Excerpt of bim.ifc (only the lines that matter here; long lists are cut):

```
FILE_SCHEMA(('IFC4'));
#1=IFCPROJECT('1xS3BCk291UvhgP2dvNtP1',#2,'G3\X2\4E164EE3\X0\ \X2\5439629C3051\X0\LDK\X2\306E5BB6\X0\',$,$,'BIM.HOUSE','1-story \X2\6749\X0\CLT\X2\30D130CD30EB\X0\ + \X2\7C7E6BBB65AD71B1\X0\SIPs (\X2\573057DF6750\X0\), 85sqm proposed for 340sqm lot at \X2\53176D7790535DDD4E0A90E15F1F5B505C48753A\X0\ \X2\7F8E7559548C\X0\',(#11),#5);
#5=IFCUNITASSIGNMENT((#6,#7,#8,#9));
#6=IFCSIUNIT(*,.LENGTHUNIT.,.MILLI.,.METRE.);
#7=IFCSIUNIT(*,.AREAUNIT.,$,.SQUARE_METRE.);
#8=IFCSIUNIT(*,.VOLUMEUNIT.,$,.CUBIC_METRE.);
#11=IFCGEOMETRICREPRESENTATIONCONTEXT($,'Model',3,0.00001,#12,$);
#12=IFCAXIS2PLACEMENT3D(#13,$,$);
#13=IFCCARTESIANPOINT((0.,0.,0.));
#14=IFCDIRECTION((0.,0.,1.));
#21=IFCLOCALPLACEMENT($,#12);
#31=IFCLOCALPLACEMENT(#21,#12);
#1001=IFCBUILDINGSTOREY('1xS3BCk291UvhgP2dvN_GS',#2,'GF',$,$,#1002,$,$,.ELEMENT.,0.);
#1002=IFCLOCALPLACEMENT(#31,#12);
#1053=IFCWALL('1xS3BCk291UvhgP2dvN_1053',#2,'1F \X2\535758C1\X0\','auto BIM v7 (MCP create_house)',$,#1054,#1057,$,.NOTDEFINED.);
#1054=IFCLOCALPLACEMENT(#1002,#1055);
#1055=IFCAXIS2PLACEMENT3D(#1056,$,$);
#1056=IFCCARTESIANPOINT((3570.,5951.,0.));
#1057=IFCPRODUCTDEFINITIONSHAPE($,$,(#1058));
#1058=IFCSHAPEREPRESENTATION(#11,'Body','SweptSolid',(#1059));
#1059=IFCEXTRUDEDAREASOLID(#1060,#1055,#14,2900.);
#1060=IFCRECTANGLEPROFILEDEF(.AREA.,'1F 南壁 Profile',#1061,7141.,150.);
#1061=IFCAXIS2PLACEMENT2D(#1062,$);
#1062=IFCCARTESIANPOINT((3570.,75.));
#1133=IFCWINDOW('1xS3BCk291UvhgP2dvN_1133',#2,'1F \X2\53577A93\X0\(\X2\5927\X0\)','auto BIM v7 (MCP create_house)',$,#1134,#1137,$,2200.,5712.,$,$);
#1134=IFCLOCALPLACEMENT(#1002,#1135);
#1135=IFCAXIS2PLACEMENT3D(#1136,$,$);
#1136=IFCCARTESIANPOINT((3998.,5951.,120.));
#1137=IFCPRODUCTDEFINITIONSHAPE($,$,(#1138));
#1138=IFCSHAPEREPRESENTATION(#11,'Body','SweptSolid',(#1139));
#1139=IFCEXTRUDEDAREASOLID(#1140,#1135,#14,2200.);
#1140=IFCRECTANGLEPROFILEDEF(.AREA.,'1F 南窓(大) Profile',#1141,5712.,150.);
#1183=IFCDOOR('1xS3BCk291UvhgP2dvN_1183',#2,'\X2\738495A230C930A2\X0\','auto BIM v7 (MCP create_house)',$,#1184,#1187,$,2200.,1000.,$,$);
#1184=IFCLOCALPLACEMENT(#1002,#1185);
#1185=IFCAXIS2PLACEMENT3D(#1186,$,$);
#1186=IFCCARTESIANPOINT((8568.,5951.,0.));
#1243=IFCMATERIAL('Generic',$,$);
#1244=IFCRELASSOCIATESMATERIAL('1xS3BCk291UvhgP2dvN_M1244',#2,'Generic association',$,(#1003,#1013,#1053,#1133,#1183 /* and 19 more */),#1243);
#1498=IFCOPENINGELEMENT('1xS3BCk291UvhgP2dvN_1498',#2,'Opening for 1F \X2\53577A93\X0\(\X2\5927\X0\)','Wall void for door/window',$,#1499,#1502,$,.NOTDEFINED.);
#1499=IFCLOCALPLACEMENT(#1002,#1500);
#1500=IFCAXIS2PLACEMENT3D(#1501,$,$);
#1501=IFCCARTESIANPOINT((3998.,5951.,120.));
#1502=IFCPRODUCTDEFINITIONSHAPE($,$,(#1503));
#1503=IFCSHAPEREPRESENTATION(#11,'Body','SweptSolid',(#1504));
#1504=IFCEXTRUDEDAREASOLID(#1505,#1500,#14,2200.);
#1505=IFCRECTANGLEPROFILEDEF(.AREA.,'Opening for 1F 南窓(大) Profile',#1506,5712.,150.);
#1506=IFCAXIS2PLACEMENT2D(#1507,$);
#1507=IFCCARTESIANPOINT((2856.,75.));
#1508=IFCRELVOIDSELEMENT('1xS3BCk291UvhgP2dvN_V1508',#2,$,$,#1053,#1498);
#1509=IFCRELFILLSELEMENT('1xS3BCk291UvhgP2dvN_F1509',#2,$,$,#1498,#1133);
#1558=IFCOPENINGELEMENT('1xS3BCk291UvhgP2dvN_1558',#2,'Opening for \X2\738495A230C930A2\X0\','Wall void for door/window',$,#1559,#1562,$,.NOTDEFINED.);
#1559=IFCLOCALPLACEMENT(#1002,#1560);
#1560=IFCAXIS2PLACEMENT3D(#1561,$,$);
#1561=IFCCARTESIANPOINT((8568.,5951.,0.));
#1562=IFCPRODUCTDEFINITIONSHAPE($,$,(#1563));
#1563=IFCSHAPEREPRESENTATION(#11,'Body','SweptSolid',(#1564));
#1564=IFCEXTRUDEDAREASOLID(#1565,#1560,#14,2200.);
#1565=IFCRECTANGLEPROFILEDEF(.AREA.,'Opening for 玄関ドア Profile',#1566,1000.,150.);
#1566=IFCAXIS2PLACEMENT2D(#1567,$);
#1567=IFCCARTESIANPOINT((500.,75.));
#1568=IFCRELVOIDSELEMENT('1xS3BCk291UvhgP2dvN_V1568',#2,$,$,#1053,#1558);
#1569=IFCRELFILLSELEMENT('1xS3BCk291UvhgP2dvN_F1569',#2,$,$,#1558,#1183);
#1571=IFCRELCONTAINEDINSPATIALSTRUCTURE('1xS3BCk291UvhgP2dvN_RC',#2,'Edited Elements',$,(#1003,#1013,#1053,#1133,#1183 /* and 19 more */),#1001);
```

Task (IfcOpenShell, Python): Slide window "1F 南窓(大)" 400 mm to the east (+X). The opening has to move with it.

```python
import ifcopenshell
import ifcopenshell.api.geometry
import ifcopenshell.util.placement

model = ifcopenshell.open("bim.ifc")

window = model.by_guid("1xS3BCk291UvhgP2dvN_1133")
opening = window.FillsVoids[0].RelatingOpeningElement
wall = opening.VoidsElements[0].RelatingBuildingElement

wall_matrix = ifcopenshell.util.placement.get_local_placement(wall.ObjectPlacement)
shift = wall_matrix[:3, 0] * 400.0
before = ifcopenshell.util.placement.get_local_placement(window.ObjectPlacement)[:3, 3].copy()

# The window is not placed relative to its opening, so move both.
for product in (opening, window):
    matrix = ifcopenshell.util.placement.get_local_placement(product.ObjectPlacement)
    matrix[:3, 3] += shift
    ifcopenshell.api.geometry.edit_object_placement(model, product=product, matrix=matrix, is_si=False)

after = ifcopenshell.util.placement.get_local_placement(window.ObjectPlacement)[:3, 3]
print("window moved by", (after - before).round(3) + 0.0)

model.write("bim_edited.ifc")
```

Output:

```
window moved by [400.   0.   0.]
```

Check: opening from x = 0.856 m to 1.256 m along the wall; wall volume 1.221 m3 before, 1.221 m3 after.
